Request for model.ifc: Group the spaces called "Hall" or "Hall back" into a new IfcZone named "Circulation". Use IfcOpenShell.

First a look at what the model holds.

```python
import ifcopenshell

model = ifcopenshell.open("model.ifc")
print(model.schema)
seen = {}
for space in model.by_type("IfcSpace"):
    seen[space.LongName] = seen.get(space.LongName, 0) + 1
for name, count in sorted(seen.items(), key=str):
    print(count, "x", name)
print("zones:", [z.Name for z in model.by_type("IfcZone")][:20])
```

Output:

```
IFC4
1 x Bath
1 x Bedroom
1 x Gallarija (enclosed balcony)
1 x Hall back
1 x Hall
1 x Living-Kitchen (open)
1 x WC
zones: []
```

```python
import ifcopenshell
import ifcopenshell.api.group
import ifcopenshell.api.root

model = ifcopenshell.open("model.ifc")

names = {"Hall", "Hall back"}
spaces = [s for s in model.by_type("IfcSpace") if s.LongName in names]

zone = ifcopenshell.api.root.create_entity(model, ifc_class="IfcZone", name="Circulation")
ifcopenshell.api.group.assign_group(model, products=spaces, group=zone)
print(len(spaces), "spaces in", zone.Name)

model.write("model_updated.ifc")
```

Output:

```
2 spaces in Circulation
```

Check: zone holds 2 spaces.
